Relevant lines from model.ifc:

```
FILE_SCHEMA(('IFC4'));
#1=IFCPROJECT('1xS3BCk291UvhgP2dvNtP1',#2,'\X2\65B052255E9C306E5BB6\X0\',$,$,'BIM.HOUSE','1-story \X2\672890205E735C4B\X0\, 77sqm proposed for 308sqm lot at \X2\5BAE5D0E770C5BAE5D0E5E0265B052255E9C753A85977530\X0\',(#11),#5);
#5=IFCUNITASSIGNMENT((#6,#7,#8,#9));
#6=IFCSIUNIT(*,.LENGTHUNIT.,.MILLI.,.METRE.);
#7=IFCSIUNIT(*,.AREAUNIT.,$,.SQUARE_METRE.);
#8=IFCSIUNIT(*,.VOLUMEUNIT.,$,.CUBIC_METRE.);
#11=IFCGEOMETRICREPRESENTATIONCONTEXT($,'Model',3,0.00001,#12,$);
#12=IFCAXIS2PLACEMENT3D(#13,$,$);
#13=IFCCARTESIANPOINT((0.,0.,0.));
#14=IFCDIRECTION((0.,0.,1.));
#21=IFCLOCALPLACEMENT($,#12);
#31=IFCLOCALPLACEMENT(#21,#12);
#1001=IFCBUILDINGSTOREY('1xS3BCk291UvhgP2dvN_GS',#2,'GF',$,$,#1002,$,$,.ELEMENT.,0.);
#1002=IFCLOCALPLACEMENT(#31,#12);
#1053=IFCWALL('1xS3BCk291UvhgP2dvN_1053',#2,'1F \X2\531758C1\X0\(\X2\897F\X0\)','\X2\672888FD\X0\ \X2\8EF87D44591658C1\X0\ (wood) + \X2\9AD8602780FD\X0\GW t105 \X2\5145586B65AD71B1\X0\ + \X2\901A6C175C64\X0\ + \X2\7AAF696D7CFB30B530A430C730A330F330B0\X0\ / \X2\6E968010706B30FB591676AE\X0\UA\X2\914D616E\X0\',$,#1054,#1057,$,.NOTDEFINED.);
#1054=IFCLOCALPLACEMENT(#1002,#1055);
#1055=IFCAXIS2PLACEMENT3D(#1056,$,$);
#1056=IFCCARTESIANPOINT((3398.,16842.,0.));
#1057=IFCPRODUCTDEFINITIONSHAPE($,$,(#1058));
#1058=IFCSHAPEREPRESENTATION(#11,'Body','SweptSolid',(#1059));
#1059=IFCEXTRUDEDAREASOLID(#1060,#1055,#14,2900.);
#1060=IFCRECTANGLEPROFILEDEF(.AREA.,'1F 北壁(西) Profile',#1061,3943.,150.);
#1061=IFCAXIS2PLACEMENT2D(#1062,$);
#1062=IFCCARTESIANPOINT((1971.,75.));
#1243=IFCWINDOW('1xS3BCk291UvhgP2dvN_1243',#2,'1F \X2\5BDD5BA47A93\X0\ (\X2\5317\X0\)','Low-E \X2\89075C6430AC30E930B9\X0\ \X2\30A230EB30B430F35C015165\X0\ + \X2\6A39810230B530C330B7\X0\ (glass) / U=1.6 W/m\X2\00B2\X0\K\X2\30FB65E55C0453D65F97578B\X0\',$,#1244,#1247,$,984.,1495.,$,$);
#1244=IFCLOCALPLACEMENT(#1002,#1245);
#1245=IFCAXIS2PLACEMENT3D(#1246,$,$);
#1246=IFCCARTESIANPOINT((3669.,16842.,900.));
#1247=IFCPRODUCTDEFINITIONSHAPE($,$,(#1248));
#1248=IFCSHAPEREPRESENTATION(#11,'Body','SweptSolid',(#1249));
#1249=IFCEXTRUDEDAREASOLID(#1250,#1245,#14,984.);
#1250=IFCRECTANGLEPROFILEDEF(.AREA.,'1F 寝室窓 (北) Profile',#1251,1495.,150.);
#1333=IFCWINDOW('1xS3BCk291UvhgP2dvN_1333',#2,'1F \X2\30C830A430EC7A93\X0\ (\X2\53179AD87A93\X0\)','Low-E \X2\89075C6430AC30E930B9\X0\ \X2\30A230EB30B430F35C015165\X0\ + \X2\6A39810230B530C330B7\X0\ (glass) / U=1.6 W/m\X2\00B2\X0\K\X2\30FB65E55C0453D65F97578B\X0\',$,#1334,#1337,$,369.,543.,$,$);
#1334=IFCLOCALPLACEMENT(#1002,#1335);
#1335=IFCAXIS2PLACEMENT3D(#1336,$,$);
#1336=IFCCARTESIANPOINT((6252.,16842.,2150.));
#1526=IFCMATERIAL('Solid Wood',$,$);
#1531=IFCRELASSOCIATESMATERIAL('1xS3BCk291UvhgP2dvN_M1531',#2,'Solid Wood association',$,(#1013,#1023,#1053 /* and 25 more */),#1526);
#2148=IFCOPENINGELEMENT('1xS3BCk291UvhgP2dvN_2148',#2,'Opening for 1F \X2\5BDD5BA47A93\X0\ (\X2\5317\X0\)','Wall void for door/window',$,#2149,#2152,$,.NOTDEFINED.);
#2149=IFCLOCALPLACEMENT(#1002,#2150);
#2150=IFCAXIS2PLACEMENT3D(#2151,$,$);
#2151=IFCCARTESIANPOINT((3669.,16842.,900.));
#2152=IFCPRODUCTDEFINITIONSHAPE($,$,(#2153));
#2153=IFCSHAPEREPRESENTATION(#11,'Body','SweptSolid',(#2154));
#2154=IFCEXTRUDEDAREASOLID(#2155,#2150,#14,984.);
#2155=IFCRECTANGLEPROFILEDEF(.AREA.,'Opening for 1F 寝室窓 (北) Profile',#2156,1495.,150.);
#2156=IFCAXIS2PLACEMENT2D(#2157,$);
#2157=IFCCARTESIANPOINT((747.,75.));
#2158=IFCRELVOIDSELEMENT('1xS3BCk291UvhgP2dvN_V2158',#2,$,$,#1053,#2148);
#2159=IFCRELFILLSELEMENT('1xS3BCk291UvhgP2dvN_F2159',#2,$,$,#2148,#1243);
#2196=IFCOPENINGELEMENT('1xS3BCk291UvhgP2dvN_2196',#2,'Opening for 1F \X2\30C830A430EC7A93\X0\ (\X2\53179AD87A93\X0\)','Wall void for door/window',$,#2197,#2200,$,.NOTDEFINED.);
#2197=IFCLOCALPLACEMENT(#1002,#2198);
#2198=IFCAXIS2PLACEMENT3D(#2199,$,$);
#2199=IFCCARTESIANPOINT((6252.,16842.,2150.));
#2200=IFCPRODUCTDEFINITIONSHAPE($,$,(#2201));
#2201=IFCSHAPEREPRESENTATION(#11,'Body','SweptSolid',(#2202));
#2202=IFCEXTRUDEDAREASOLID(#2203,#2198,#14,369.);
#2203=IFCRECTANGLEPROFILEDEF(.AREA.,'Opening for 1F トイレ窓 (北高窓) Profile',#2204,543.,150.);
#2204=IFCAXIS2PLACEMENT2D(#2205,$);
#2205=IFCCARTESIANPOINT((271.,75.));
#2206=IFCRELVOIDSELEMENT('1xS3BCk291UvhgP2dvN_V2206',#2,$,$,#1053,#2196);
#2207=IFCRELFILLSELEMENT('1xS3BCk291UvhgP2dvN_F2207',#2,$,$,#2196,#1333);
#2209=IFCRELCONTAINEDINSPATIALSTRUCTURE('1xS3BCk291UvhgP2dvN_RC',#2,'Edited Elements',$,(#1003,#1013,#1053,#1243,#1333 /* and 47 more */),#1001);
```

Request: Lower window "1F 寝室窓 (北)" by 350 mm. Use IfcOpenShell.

```python
import numpy as np
import ifcopenshell
import ifcopenshell.api.geometry
import ifcopenshell.util.placement
import ifcopenshell.util.unit

model = ifcopenshell.open("model.ifc")
unit_scale = ifcopenshell.util.unit.calculate_unit_scale(model)

window = model.by_guid("1xS3BCk291UvhgP2dvN_1243")
opening = window.FillsVoids[0].RelatingOpeningElement
dz = -0.35 / unit_scale

shift = np.array([0.0, 0.0, dz])
# The window is not placed relative to its opening, so move both.
for product in (opening, window):
    matrix = ifcopenshell.util.placement.get_local_placement(product.ObjectPlacement)
    matrix[:3, 3] += shift
    ifcopenshell.api.geometry.edit_object_placement(model, product=product, matrix=matrix, is_si=False)

print(f"moved by {dz * unit_scale:+.3f} m")

model.write("model_rev.ifc")
```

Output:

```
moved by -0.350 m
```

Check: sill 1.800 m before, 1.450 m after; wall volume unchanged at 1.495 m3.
